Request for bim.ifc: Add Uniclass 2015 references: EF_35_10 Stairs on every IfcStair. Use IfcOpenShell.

First a look at what the model holds.

```python
import ifcopenshell

model = ifcopenshell.open("bim.ifc")
print(model.schema)
print("classifications:", [c.Name for c in model.by_type("IfcClassification")])
for ifc_class in ("IfcDoor", "IfcRoof", "IfcStair", "IfcWall", "IfcWindow"):
    print(ifc_class, len(model.by_type(ifc_class)))
```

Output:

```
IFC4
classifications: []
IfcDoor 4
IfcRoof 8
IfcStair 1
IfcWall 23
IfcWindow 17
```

```python
import ifcopenshell
import ifcopenshell.api.classification

model = ifcopenshell.open("bim.ifc")

system = ifcopenshell.api.classification.add_classification(model, classification="Uniclass 2015")

codes = {
    "IfcStair": ("EF_35_10", "Stairs"),
}
for ifc_class, (code, name) in codes.items():
    products = model.by_type(ifc_class)
    ifcopenshell.api.classification.add_reference(
        model, products=products, classification=system, identification=code, name=name
    )
    print(code, len(products))

model.write("bim_v2.ifc")
```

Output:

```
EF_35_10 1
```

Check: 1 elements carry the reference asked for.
